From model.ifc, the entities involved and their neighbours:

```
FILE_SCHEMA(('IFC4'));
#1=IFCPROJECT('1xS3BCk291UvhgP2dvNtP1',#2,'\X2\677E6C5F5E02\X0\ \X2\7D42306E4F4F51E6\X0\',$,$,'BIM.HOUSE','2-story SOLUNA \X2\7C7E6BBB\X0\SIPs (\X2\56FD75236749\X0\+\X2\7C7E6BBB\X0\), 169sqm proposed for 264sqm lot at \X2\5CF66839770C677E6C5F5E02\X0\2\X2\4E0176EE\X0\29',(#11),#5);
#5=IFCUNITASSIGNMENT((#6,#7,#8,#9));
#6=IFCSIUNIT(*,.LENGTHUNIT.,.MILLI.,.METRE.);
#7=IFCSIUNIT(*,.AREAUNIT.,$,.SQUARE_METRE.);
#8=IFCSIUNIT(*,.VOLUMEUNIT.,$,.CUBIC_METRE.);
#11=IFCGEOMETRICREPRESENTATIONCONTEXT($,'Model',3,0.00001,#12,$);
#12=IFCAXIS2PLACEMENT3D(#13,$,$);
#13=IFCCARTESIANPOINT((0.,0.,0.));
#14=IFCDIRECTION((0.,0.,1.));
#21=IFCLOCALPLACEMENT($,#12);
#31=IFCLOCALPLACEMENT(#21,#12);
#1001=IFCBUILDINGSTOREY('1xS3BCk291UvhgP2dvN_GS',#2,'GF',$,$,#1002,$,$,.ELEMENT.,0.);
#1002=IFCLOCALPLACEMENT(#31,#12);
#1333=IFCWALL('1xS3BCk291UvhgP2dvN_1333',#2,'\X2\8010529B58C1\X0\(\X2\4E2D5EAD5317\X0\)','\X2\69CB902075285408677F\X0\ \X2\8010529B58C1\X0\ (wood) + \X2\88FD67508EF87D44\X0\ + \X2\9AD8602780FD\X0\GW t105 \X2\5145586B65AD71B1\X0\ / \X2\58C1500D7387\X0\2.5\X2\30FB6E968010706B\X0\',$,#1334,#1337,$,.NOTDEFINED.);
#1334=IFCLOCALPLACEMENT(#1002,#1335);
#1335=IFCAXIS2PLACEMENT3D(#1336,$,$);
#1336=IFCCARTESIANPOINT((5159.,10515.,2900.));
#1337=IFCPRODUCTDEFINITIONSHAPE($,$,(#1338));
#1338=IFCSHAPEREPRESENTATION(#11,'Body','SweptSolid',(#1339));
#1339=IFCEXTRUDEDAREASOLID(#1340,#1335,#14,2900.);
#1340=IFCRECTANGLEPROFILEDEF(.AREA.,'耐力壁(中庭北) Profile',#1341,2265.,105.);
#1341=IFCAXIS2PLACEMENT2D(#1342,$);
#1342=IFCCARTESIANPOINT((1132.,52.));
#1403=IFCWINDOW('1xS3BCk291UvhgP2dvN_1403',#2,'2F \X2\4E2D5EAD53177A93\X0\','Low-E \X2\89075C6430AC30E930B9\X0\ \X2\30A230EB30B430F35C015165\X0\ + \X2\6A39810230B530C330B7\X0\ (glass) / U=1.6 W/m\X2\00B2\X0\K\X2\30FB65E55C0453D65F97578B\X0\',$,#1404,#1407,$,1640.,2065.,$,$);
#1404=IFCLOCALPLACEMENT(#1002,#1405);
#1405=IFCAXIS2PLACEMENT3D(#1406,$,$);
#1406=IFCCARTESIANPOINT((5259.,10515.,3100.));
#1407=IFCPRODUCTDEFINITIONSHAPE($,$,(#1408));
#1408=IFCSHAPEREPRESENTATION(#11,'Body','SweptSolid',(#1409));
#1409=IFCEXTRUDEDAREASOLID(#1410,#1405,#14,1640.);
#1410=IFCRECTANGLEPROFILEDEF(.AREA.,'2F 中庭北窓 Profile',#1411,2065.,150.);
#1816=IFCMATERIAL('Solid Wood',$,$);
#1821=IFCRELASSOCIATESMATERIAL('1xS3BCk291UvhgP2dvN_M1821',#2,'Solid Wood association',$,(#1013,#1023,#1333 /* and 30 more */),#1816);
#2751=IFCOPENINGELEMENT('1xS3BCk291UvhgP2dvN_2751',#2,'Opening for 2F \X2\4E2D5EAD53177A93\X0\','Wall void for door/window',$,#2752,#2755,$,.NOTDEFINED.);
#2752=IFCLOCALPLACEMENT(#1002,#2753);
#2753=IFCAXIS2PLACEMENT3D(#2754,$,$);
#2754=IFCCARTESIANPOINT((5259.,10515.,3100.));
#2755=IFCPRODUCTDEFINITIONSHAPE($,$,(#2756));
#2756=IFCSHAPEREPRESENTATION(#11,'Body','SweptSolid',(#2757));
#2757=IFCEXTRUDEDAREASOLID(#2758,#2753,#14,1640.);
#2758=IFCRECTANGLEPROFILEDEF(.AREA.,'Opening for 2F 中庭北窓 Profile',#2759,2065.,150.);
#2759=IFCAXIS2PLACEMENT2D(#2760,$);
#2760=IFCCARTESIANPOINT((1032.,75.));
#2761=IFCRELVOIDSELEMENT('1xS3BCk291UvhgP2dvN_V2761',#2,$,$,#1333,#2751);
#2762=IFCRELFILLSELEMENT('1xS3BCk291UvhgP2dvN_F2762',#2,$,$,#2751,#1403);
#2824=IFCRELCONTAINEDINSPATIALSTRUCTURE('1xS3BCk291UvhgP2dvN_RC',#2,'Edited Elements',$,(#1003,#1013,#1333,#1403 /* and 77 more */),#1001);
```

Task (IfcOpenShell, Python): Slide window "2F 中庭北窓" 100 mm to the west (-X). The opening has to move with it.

```python
import ifcopenshell
import ifcopenshell.api.geometry
import ifcopenshell.util.placement

model = ifcopenshell.open("model.ifc")

window = model.by_guid("1xS3BCk291UvhgP2dvN_1403")
opening = window.FillsVoids[0].RelatingOpeningElement
wall = opening.VoidsElements[0].RelatingBuildingElement

wall_matrix = ifcopenshell.util.placement.get_local_placement(wall.ObjectPlacement)
shift = wall_matrix[:3, 0] * -100.0
before = ifcopenshell.util.placement.get_local_placement(window.ObjectPlacement)[:3, 3].copy()

# The window is not placed relative to its opening, so move both.
for product in (opening, window):
    matrix = ifcopenshell.util.placement.get_local_placement(product.ObjectPlacement)
    matrix[:3, 3] += shift
    ifcopenshell.api.geometry.edit_object_placement(model, product=product, matrix=matrix, is_si=False)

after = ifcopenshell.util.placement.get_local_placement(window.ObjectPlacement)[:3, 3]
print("window moved by", (after - before).round(3) + 0.0)

model.write("model-out.ifc")
```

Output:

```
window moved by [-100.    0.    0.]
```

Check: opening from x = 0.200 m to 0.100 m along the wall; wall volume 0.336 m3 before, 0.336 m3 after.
